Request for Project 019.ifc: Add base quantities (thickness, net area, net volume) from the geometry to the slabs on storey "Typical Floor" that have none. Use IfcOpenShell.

First a look at what the model holds.

```python
import ifcopenshell
import ifcopenshell.util.element
import ifcopenshell.util.unit

model = ifcopenshell.open("Project 019.ifc")
print(model.schema)
for unit_type in ("LENGTHUNIT", "AREAUNIT", "VOLUMEUNIT"):
    print(unit_type, ifcopenshell.util.unit.calculate_unit_scale(model, unit_type))
storey = next(s for s in model.by_type("IfcBuildingStorey") if s.Name == "Typical Floor")
slabs = [e for e in ifcopenshell.util.element.get_decomposition(storey) if e.is_a("IfcSlab")]
for e in sorted(slabs, key=lambda e: e.id()):
    print(e.id(), e.is_a(), e.Name, list(ifcopenshell.util.element.get_psets(e, qtos_only=True)), sep=" | ")
```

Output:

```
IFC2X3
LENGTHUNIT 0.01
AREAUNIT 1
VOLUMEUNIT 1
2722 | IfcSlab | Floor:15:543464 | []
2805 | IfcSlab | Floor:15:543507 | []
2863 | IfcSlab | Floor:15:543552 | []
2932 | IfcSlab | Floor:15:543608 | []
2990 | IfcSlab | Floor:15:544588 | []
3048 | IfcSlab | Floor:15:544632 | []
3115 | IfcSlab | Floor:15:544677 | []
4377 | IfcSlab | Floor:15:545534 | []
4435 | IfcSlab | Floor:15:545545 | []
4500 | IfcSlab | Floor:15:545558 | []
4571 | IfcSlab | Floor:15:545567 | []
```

```python
import ifcopenshell
import ifcopenshell.api.pset
import ifcopenshell.geom
import ifcopenshell.util.element
import ifcopenshell.util.shape
import ifcopenshell.util.unit

model = ifcopenshell.open("Project 019.ifc")
unit_scale = ifcopenshell.util.unit.calculate_unit_scale(model)
area_scale = ifcopenshell.util.unit.calculate_unit_scale(model, "AREAUNIT")
volume_scale = ifcopenshell.util.unit.calculate_unit_scale(model, "VOLUMEUNIT")
settings = ifcopenshell.geom.settings()

storey = next(s for s in model.by_type("IfcBuildingStorey") if s.Name == "Typical Floor")
slabs = [e for e in ifcopenshell.util.element.get_decomposition(storey) if e.is_a("IfcSlab")]

for e in sorted(slabs, key=lambda e: e.id()):
    if ifcopenshell.util.element.get_psets(e, qtos_only=True, should_inherit=False):
        continue
    # Geometry comes back in metres, in the element's own axes.
    shape = ifcopenshell.geom.create_shape(settings, e)
    values = {
        "Width": ifcopenshell.util.shape.get_z(shape.geometry) / unit_scale,
        "NetArea": ifcopenshell.util.shape.get_footprint_area(shape.geometry) / area_scale,
        "NetVolume": ifcopenshell.util.shape.get_volume(shape.geometry) / volume_scale,
    }
    qto = ifcopenshell.api.pset.add_qto(model, product=e, name="BaseQuantities")
    ifcopenshell.api.pset.edit_qto(model, qto=qto, properties=values)
    print(e.id(), {k: round(v, 3) for k, v in values.items()})

model.write("Project 019_updated.ifc")
```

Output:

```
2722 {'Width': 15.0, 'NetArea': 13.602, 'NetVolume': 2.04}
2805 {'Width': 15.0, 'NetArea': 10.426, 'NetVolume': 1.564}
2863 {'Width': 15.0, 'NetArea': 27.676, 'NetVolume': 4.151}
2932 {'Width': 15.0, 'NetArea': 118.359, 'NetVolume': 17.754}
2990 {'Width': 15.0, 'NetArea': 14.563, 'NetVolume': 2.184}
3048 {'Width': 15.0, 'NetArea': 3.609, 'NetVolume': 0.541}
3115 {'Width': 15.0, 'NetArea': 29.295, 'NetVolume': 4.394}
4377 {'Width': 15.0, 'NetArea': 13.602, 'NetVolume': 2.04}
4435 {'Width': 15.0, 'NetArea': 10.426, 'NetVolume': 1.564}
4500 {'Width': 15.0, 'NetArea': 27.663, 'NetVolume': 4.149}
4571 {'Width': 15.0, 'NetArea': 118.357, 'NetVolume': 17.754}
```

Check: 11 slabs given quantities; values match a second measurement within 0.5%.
